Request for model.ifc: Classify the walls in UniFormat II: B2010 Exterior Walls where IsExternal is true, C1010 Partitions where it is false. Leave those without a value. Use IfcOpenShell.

First a look at what the model holds.

```python
import ifcopenshell
import ifcopenshell.util.element

model = ifcopenshell.open("model.ifc")
print(model.schema)
print("classifications:", [c.Name for c in model.by_type("IfcClassification")])
values = [ifcopenshell.util.element.get_pset(e, "Pset_WallCommon", "IsExternal") for e in model.by_type("IfcWall")]
for value in (True, False, None):
    print("IsExternal", value, values.count(value))
```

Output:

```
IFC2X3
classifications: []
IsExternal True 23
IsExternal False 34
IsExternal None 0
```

```python
import ifcopenshell
import ifcopenshell.api.classification
import ifcopenshell.util.element

model = ifcopenshell.open("model.ifc")

# IFC2X3 requires Source and Edition and has no link from the project to the system.
system = model.create_entity("IfcClassification", Source="ASTM", Edition="E1557", Name="UniFormat II")

walls = model.by_type("IfcWall")
external = {e: ifcopenshell.util.element.get_pset(e, "Pset_WallCommon", "IsExternal") for e in walls}
for flag, code, name in ((True, "B2010", "Exterior Walls"), (False, "C1010", "Partitions")):
    products = [e for e in walls if external[e] is flag]
    ifcopenshell.api.classification.add_reference(
        model, products=products, classification=system, identification=code, name=name
    )
    print(code, len(products))

model.write("model-out.ifc")
```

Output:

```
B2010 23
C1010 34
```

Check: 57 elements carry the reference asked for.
